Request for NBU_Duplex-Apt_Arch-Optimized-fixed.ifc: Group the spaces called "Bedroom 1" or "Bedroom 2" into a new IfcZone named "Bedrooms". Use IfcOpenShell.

First a look at what the model holds.

```python
import ifcopenshell

model = ifcopenshell.open("NBU_Duplex-Apt_Arch-Optimized-fixed.ifc")
print(model.schema)
seen = {}
for space in model.by_type("IfcSpace"):
    seen[space.LongName] = seen.get(space.LongName, 0) + 1
for name, count in sorted(seen.items(), key=str):
    print(count, "x", name)
print("zones:", [z.Name for z in model.by_type("IfcZone")][:20])
```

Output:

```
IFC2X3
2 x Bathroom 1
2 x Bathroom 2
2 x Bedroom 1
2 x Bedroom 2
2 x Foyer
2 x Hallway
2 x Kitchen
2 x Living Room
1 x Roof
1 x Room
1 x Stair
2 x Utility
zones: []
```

```python
import ifcopenshell
import ifcopenshell.api.group
import ifcopenshell.api.root

model = ifcopenshell.open("NBU_Duplex-Apt_Arch-Optimized-fixed.ifc")

names = {"Bedroom 1", "Bedroom 2"}
spaces = [s for s in model.by_type("IfcSpace") if s.LongName in names]

zone = ifcopenshell.api.root.create_entity(model, ifc_class="IfcZone", name="Bedrooms")
ifcopenshell.api.group.assign_group(model, products=spaces, group=zone)
print(len(spaces), "spaces in", zone.Name)

model.write("NBU_Duplex-Apt_Arch-Optimized-fixed_rev.ifc")
```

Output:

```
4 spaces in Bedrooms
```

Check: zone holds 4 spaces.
